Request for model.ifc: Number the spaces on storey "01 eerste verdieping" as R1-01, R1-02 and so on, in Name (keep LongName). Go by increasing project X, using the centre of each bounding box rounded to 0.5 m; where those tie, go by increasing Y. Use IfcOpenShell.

First a look at what the model holds.

```python
import ifcopenshell
import ifcopenshell.util.element
import ifcopenshell.util.placement

model = ifcopenshell.open("model.ifc")
print(model.schema)
storey = next(s for s in model.by_type("IfcBuildingStorey") if s.Name == "01 eerste verdieping")
spaces = [e for e in ifcopenshell.util.element.get_decomposition(storey) if e.is_a("IfcSpace")]
for e in sorted(spaces, key=lambda e: e.id()):
    origin = ifcopenshell.util.placement.get_local_placement(e.ObjectPlacement)[:3, 3]
    print(e.id(), e.Name, e.LongName, origin.round(2) + 0.0, sep=" | ")
```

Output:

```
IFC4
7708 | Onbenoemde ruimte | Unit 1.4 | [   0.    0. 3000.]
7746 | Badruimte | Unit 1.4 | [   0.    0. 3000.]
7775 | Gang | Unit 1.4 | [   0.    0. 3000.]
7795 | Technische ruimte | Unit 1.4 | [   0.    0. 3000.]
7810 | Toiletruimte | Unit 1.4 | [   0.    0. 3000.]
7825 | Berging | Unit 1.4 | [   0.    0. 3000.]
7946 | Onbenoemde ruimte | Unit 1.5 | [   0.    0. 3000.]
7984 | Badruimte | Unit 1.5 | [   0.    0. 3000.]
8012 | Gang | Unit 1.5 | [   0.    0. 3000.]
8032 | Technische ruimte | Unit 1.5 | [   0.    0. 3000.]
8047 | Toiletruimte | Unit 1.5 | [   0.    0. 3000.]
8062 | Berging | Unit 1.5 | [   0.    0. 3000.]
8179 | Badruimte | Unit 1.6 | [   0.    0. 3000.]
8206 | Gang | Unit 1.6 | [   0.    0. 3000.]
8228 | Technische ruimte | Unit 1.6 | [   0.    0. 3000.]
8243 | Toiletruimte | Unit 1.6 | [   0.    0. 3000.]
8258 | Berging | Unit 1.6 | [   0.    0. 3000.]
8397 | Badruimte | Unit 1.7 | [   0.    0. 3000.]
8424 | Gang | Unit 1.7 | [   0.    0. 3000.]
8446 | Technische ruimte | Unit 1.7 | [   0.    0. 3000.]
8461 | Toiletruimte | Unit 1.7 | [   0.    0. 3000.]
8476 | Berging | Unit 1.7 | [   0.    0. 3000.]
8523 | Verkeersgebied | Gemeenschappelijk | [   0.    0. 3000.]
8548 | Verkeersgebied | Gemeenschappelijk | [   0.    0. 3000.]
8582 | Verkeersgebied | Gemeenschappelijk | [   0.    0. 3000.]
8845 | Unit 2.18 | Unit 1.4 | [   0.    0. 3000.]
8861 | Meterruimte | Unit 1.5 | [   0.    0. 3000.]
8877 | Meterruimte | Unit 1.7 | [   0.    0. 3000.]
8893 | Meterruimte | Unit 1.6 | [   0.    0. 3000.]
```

```python
import ifcopenshell
import ifcopenshell.geom
import ifcopenshell.util.element
import ifcopenshell.util.shape

model = ifcopenshell.open("model.ifc")
settings = ifcopenshell.geom.settings()
settings.set("use-world-coords", True)


def centre(element):
    shape = ifcopenshell.geom.create_shape(settings, element)
    return ifcopenshell.util.shape.get_bbox_centroid(shape.geometry)


storey = next(s for s in model.by_type("IfcBuildingStorey") if s.Name == "01 eerste verdieping")
spaces = [e for e in ifcopenshell.util.element.get_decomposition(storey) if e.is_a("IfcSpace")]

# Insertion points can sit at a corner or the storey origin, so sort by the geometry (in metres).
centres = {e: centre(e) for e in spaces}
spaces.sort(key=lambda e: (round(centres[e][0] / 0.5), centres[e][1]))

for i, e in enumerate(spaces, start=1):
    number = f"R1-{i:02d}"
    e.Name = number
    print(e.id(), number)

model.write("model_rev.ifc")
```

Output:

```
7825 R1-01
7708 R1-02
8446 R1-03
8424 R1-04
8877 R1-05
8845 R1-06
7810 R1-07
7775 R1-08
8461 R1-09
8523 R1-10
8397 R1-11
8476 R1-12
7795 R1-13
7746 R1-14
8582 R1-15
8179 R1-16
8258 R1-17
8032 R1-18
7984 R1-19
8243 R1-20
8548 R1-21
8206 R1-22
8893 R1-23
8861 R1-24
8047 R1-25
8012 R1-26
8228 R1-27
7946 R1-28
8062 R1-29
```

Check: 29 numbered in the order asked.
